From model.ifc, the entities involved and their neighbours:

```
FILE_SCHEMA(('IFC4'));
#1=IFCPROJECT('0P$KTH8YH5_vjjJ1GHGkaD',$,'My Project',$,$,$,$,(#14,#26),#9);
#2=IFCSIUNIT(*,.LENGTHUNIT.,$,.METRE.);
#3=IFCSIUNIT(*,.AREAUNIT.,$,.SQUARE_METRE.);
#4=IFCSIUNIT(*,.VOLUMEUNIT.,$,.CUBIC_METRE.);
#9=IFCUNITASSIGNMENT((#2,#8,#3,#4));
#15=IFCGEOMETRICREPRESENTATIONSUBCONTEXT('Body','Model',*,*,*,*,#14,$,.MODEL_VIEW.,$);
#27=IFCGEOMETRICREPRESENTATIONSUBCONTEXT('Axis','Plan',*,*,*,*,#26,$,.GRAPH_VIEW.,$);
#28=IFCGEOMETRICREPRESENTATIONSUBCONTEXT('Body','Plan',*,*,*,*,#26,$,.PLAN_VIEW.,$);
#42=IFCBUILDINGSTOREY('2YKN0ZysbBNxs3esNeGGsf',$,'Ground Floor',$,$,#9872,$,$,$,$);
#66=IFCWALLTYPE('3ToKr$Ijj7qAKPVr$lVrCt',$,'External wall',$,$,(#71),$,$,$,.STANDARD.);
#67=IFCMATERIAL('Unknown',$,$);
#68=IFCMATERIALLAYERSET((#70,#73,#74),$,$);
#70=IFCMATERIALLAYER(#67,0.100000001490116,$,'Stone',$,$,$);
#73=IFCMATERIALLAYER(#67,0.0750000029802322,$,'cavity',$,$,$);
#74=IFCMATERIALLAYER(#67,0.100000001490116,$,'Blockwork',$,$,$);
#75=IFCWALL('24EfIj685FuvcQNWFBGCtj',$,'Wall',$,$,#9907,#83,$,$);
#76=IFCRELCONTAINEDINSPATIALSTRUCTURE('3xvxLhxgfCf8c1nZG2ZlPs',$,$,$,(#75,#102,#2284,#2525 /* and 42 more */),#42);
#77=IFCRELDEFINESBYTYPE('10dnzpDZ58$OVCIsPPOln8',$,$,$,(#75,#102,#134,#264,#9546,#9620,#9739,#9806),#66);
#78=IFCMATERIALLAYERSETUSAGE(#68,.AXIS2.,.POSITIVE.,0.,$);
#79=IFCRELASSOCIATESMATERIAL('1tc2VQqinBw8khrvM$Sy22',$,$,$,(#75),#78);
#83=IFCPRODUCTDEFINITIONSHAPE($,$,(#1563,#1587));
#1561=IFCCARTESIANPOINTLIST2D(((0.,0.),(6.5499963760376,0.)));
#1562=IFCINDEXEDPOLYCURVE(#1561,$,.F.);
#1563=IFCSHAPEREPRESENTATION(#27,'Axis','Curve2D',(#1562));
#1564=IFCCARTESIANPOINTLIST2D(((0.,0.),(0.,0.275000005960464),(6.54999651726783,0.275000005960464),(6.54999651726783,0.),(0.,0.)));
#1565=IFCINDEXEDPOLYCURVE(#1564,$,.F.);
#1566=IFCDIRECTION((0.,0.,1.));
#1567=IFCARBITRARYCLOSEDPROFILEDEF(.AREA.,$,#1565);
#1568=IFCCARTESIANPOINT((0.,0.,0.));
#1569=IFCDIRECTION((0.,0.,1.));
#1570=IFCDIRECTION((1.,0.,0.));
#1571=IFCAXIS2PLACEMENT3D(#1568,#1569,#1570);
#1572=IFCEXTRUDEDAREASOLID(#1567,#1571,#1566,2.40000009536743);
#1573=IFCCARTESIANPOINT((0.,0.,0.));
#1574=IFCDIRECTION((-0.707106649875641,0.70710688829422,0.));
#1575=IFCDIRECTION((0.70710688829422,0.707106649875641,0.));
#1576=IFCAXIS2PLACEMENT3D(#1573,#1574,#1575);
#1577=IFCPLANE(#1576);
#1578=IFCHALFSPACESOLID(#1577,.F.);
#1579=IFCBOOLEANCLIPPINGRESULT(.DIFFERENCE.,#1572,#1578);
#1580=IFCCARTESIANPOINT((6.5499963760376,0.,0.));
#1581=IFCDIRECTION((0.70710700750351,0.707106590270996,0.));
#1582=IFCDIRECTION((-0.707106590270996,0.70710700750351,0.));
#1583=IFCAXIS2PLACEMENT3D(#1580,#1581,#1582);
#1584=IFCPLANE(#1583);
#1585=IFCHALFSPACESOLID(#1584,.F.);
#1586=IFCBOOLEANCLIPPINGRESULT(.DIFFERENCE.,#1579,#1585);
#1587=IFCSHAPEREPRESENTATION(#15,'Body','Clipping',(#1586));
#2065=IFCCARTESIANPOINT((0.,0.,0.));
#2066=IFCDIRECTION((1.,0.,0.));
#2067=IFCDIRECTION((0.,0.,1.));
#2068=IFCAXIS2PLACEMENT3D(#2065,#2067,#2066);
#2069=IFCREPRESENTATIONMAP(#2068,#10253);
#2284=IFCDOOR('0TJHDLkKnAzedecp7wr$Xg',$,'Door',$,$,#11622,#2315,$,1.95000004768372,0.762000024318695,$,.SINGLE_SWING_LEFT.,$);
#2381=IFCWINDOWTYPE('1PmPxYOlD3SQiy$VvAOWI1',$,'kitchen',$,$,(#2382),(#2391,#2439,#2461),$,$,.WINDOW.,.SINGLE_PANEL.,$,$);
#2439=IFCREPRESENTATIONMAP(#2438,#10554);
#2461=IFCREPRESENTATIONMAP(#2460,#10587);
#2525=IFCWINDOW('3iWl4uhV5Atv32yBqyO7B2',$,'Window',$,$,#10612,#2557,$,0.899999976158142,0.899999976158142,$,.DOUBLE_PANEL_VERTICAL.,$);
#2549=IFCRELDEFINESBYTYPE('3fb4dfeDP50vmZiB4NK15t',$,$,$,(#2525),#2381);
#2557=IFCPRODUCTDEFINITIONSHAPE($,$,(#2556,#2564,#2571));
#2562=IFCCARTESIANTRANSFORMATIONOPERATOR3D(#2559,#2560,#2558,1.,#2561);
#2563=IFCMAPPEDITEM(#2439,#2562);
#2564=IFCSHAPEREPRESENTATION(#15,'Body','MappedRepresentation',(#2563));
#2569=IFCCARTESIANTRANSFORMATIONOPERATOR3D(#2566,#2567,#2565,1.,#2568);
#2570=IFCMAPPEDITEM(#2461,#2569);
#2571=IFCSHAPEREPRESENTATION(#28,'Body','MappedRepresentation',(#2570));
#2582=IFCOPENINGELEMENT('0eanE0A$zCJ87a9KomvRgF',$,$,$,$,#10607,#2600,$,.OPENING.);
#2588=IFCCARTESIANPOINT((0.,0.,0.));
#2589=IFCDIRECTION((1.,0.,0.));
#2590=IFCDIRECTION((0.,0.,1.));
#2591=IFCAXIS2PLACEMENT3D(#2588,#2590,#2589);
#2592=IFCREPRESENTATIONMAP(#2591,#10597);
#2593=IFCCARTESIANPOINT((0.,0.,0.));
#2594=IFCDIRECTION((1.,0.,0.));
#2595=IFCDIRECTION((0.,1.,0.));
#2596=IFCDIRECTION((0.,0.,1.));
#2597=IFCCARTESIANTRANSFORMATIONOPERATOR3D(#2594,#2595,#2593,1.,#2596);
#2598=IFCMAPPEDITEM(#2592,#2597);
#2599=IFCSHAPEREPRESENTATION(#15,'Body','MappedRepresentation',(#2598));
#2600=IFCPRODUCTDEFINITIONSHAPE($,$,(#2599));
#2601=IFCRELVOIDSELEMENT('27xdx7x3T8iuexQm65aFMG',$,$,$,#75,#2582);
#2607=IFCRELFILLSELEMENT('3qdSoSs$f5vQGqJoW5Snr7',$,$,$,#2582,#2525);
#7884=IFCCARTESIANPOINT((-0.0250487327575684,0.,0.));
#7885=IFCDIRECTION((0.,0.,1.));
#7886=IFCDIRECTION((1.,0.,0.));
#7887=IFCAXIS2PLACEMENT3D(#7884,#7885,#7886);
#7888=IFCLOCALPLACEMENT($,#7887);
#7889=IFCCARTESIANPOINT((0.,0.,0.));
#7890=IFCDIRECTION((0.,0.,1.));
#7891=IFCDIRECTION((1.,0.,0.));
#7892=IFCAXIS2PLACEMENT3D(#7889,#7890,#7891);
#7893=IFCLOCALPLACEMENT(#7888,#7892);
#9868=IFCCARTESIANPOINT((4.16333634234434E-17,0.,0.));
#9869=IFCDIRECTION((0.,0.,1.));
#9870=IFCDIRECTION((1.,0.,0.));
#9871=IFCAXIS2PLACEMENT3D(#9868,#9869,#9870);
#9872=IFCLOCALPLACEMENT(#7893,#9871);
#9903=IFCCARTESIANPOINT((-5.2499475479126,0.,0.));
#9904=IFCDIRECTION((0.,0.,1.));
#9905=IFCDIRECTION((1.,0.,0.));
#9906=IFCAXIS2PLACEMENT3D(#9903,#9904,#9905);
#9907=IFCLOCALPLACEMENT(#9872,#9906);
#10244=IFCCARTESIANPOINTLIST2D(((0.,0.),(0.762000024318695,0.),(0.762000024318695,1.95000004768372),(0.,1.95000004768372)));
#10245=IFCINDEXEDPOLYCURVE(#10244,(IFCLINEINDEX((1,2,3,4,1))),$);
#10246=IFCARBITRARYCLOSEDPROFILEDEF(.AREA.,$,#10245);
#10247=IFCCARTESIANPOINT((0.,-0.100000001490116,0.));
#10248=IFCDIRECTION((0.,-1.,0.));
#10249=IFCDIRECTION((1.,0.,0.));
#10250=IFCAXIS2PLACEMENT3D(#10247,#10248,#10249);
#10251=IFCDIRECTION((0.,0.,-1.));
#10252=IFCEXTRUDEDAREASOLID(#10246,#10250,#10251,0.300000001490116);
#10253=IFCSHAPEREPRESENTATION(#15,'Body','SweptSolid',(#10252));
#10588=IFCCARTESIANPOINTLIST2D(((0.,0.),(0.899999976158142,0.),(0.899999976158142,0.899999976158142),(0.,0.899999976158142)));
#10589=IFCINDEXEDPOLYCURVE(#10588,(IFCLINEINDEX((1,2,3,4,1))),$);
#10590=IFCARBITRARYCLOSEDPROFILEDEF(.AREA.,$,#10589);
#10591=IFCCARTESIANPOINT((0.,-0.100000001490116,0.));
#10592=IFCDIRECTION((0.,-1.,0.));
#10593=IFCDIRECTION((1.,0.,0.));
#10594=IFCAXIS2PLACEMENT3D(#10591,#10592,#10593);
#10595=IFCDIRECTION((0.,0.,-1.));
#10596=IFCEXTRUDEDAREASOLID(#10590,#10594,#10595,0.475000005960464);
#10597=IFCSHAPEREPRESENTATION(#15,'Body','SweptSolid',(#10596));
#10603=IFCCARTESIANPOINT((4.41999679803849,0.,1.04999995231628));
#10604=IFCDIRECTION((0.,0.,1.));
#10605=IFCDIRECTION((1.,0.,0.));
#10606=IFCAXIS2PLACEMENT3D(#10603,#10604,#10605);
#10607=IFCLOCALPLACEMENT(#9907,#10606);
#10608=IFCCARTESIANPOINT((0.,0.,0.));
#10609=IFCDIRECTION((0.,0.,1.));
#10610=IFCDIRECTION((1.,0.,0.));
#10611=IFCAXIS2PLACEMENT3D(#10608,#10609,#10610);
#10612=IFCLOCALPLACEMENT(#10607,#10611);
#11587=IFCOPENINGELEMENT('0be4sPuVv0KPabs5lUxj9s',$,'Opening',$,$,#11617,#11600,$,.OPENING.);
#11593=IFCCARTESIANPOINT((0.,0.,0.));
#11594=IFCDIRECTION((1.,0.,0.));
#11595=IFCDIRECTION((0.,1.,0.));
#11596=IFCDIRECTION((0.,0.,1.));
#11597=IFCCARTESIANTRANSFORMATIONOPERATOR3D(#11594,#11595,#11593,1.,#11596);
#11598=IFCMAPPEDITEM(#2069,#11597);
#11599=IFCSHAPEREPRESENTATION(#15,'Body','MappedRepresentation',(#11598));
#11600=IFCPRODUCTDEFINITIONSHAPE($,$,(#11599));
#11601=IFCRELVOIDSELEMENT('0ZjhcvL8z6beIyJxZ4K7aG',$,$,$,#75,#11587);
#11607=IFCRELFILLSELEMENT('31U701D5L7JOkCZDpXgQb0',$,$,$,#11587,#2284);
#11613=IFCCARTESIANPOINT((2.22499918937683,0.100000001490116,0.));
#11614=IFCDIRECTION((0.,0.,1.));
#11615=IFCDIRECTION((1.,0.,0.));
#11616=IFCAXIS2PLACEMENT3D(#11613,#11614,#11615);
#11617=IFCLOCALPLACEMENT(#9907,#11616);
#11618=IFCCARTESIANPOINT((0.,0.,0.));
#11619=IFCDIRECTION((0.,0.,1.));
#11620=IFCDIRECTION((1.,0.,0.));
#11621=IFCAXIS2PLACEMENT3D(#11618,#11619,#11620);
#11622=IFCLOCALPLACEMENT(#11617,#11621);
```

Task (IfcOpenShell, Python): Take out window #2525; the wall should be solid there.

```python
import ifcopenshell
import ifcopenshell.api.feature
import ifcopenshell.api.root
import ifcopenshell.geom
import ifcopenshell.util.shape

model = ifcopenshell.open("model.ifc")
settings = ifcopenshell.geom.settings()


def volume(element):
    """Net volume in cubic metres, openings subtracted."""
    shape = ifcopenshell.geom.create_shape(settings, element)
    return ifcopenshell.util.shape.get_volume(shape.geometry)


window = model.by_guid("3iWl4uhV5Atv32yBqyO7B2")
opening = window.FillsVoids[0].RelatingOpeningElement
wall = opening.VoidsElements[0].RelatingBuildingElement
before = volume(wall)

ifcopenshell.api.root.remove_product(model, product=window)
ifcopenshell.api.feature.remove_feature(model, feature=opening)

after = volume(wall)

print(f"wall volume {before:.3f} -> {after:.3f} m3")

model.write("model_rev.ifc")
```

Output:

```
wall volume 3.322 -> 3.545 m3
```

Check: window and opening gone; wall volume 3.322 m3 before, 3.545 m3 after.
